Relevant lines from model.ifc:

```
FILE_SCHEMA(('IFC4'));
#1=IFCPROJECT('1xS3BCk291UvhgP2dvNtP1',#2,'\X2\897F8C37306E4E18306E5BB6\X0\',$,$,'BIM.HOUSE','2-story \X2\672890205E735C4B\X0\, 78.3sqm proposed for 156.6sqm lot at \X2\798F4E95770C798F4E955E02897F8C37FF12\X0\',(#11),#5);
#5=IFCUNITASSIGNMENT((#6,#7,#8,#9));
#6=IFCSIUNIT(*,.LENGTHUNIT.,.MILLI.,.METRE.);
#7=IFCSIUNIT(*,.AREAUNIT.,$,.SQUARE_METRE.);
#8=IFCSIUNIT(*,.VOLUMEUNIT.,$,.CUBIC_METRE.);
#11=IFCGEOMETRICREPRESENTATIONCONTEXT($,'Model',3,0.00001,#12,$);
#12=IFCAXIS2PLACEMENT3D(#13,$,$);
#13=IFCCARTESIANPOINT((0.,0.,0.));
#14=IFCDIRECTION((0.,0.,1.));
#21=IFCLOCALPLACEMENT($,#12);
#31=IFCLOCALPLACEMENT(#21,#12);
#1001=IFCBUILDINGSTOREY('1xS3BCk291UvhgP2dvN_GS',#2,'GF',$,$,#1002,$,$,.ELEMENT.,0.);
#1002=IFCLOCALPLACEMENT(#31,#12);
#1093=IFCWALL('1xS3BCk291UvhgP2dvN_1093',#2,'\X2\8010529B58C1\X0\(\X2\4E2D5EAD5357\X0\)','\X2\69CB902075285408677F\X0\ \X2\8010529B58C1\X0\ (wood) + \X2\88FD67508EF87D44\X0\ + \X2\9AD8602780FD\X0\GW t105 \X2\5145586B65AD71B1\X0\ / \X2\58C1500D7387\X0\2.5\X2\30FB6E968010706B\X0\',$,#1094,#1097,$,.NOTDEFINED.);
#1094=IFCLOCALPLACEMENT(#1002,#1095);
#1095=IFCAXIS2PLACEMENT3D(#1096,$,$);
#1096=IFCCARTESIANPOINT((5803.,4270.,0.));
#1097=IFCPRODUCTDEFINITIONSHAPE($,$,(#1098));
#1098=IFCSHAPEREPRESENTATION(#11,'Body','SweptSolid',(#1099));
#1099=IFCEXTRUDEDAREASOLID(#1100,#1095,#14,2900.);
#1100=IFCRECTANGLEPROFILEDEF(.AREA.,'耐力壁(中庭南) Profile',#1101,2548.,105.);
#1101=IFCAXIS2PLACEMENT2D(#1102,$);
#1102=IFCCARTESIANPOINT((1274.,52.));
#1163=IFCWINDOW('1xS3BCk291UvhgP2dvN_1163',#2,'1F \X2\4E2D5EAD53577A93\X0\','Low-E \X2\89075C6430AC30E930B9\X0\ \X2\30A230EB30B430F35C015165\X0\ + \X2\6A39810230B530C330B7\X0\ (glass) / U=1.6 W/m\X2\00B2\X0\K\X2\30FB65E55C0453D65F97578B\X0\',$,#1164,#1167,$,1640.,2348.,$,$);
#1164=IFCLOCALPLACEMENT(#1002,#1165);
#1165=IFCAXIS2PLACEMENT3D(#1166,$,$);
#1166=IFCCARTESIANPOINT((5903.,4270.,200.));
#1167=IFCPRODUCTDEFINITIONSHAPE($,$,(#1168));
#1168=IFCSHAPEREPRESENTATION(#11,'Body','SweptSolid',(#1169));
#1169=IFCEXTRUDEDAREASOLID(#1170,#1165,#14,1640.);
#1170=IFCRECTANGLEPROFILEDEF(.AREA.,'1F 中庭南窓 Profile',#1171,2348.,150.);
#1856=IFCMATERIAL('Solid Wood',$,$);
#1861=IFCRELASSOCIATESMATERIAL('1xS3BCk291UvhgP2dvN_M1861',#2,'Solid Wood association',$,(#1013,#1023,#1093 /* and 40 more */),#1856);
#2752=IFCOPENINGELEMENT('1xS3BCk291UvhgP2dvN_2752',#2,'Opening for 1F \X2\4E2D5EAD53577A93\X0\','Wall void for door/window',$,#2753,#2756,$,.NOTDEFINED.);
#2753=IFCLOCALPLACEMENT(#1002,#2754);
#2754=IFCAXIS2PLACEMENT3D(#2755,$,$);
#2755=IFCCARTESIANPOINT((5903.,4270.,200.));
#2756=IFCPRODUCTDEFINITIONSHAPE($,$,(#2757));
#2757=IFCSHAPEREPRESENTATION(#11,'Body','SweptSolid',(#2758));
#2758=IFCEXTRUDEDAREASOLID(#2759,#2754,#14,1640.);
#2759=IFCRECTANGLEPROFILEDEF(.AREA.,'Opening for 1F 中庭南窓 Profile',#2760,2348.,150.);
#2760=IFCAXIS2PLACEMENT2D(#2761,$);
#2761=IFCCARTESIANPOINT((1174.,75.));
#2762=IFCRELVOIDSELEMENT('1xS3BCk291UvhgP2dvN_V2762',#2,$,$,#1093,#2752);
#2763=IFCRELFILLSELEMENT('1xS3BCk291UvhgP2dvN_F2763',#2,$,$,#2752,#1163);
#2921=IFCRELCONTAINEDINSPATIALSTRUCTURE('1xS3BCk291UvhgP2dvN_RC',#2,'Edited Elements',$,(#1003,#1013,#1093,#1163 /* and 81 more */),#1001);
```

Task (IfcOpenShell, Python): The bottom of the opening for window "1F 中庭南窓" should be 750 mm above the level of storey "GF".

```python
import numpy as np
import ifcopenshell
import ifcopenshell.api.geometry
import ifcopenshell.geom
import ifcopenshell.util.element
import ifcopenshell.util.placement
import ifcopenshell.util.shape
import ifcopenshell.util.unit

model = ifcopenshell.open("model.ifc")
unit_scale = ifcopenshell.util.unit.calculate_unit_scale(model)

window = model.by_id(1163)
opening = window.FillsVoids[0].RelatingOpeningElement
storey = ifcopenshell.util.element.get_container(window, ifc_class="IfcBuildingStorey")
level = ifcopenshell.util.placement.get_local_placement(storey.ObjectPlacement)[2, 3]

# The opening's origin need not be at the sill, so measure its lowest point.
shape = ifcopenshell.geom.create_shape(ifcopenshell.geom.settings(), opening)
bottom = ifcopenshell.util.shape.get_shape_bottom_elevation(shape, shape.geometry) / unit_scale
dz = level + 0.75 / unit_scale - bottom

shift = np.array([0.0, 0.0, dz])
# The window is not placed relative to its opening, so move both.
for product in (opening, window):
    matrix = ifcopenshell.util.placement.get_local_placement(product.ObjectPlacement)
    matrix[:3, 3] += shift
    ifcopenshell.api.geometry.edit_object_placement(model, product=product, matrix=matrix, is_si=False)

print(f"moved by {dz * unit_scale:+.3f} m")

model.write("model_edited.ifc")
```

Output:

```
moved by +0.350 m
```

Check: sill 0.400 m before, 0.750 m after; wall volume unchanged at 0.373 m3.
